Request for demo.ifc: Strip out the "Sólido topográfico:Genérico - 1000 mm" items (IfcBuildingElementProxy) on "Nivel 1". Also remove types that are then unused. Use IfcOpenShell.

First a look at what the model holds.

```python
import ifcopenshell
import ifcopenshell.util.element

model = ifcopenshell.open("demo.ifc")
print(model.schema)
storey = next(s for s in model.by_type("IfcBuildingStorey") if s.Name == "Nivel 1")
proxies = [e for e in ifcopenshell.util.element.get_decomposition(storey) if e.is_a("IfcBuildingElementProxy")]
seen = {}
for e in proxies:
    element_type = ifcopenshell.util.element.get_type(e)
    name = element_type.Name if element_type not in (None, e) else None
    seen[name] = seen.get(name, 0) + 1
for name, count in sorted(seen.items(), key=str):
    print(count, "x", name)
```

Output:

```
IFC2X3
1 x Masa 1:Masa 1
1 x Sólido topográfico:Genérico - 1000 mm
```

```python
import ifcopenshell
import ifcopenshell.api.root
import ifcopenshell.util.element

model = ifcopenshell.open("demo.ifc")

storey = next(s for s in model.by_type("IfcBuildingStorey") if s.Name == "Nivel 1")
proxies = [e for e in ifcopenshell.util.element.get_decomposition(storey) if e.is_a("IfcBuildingElementProxy")]
targets = [e for e in proxies if (t := ifcopenshell.util.element.get_type(e)) not in (None, e) and t.Name == 'Sólido topográfico:Genérico - 1000\xa0mm']
types = {ifcopenshell.util.element.get_type(e) for e in targets} - {None, *targets}

for e in targets:
    ifcopenshell.api.root.remove_product(model, product=e)
print(len(targets), "removed")

unused = [t for t in types if not ifcopenshell.util.element.get_types(t)]
for t in unused:
    ifcopenshell.api.root.remove_product(model, product=t)
print(len(unused), "unused types removed")

model.write("demo_rev.ifc")
```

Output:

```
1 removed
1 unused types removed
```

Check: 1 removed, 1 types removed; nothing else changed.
